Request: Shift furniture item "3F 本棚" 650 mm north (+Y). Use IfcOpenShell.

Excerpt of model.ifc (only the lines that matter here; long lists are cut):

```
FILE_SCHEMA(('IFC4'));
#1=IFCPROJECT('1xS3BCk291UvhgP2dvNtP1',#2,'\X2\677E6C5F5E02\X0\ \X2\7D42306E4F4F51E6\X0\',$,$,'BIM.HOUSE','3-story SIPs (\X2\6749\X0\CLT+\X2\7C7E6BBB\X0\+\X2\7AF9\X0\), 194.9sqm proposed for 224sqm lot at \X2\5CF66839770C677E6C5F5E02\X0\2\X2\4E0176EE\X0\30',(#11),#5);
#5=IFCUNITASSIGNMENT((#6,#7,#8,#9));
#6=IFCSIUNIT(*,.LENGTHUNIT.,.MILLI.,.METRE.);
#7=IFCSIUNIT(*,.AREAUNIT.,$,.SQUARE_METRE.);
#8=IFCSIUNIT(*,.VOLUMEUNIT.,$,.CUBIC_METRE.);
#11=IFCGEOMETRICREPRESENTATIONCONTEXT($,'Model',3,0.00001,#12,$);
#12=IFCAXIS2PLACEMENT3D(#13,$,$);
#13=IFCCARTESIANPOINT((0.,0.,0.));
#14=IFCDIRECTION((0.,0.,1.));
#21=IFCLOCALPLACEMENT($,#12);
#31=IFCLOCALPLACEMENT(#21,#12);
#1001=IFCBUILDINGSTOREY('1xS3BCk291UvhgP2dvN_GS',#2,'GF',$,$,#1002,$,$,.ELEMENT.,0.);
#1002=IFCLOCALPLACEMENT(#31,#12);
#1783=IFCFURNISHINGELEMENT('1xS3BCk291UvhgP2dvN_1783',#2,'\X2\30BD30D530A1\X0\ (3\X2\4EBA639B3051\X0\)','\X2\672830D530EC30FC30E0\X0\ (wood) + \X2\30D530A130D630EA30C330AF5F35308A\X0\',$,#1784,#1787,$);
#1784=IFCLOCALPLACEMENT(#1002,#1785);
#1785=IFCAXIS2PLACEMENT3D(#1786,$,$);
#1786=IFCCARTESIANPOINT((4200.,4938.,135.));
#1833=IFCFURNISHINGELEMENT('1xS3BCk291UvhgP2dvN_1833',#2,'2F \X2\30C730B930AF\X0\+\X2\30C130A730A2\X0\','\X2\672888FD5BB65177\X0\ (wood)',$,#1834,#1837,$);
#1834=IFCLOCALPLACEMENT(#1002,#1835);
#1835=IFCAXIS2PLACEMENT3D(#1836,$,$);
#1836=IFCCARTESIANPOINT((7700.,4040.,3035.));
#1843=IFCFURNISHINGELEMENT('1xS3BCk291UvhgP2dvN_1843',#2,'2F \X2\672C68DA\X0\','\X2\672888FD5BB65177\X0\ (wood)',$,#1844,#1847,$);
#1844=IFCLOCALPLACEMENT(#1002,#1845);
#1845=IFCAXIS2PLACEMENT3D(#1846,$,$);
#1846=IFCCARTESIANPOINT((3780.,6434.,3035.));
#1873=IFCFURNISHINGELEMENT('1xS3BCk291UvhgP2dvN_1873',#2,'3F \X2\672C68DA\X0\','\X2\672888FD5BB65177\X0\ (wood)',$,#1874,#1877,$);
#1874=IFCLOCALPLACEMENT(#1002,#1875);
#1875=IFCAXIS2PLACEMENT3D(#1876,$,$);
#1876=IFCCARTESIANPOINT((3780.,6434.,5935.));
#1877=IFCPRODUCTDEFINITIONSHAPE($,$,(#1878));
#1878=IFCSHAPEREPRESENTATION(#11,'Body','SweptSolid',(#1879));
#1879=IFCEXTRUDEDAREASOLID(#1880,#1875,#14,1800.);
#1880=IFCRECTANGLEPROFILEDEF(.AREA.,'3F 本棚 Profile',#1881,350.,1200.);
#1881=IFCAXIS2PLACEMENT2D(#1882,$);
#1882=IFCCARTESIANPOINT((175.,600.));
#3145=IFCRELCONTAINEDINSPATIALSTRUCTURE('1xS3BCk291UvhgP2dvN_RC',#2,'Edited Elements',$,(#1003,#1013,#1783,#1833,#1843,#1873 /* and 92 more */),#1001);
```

```python
import ifcopenshell
import ifcopenshell.api.geometry
import ifcopenshell.util.placement

model = ifcopenshell.open("model.ifc")

item = model.by_guid("1xS3BCk291UvhgP2dvN_1873")
matrix = ifcopenshell.util.placement.get_local_placement(item.ObjectPlacement)
matrix[1, 3] += 650.0
ifcopenshell.api.geometry.edit_object_placement(model, product=item, matrix=matrix, is_si=False)

print(ifcopenshell.util.placement.get_local_placement(item.ObjectPlacement).round(3) + 0.0)

model.write("model_v2.ifc")
```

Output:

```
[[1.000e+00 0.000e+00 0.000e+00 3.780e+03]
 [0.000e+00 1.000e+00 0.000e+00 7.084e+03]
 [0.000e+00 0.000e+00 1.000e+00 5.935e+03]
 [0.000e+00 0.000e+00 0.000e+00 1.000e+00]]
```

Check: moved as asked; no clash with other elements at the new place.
